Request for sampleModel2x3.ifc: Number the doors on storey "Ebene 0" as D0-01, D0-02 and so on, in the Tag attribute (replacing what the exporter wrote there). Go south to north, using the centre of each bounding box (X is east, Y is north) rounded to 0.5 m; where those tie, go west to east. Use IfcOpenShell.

First a look at what the model holds.

```python
import ifcopenshell
import ifcopenshell.util.element
import ifcopenshell.util.placement

model = ifcopenshell.open("sampleModel2x3.ifc")
print(model.schema)
storey = next(s for s in model.by_type("IfcBuildingStorey") if s.Name == "Ebene 0")
doors = [e for e in ifcopenshell.util.element.get_decomposition(storey) if e.is_a("IfcDoor")]
for e in sorted(doors, key=lambda e: e.id()):
    origin = ifcopenshell.util.placement.get_local_placement(e.ObjectPlacement)[:3, 3]
    print(e.id(), e.Tag, e.Name, origin.round(2) + 0.0, sep=" | ")
```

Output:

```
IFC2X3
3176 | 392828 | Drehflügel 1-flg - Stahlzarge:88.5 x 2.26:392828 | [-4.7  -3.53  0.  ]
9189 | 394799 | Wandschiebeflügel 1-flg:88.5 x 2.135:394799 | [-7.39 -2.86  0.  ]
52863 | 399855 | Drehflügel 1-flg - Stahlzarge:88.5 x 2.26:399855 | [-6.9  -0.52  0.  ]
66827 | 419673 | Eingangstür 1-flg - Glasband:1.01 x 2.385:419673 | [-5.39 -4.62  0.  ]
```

```python
import ifcopenshell
import ifcopenshell.geom
import ifcopenshell.util.element
import ifcopenshell.util.shape

model = ifcopenshell.open("sampleModel2x3.ifc")
settings = ifcopenshell.geom.settings()
settings.set("use-world-coords", True)


def centre(element):
    shape = ifcopenshell.geom.create_shape(settings, element)
    return ifcopenshell.util.shape.get_bbox_centroid(shape.geometry)


storey = next(s for s in model.by_type("IfcBuildingStorey") if s.Name == "Ebene 0")
doors = [e for e in ifcopenshell.util.element.get_decomposition(storey) if e.is_a("IfcDoor")]

# Insertion points can sit at a corner or the storey origin, so sort by the geometry (in metres).
centres = {e: centre(e) for e in doors}
doors.sort(key=lambda e: (round(centres[e][1] / 0.5), centres[e][0]))

for i, e in enumerate(doors, start=1):
    number = f"D0-{i:02d}"
    e.Tag = number
    print(e.id(), number)

model.write("sampleModel2x3_v2.ifc")
```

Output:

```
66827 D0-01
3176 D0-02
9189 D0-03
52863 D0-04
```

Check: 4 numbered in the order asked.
